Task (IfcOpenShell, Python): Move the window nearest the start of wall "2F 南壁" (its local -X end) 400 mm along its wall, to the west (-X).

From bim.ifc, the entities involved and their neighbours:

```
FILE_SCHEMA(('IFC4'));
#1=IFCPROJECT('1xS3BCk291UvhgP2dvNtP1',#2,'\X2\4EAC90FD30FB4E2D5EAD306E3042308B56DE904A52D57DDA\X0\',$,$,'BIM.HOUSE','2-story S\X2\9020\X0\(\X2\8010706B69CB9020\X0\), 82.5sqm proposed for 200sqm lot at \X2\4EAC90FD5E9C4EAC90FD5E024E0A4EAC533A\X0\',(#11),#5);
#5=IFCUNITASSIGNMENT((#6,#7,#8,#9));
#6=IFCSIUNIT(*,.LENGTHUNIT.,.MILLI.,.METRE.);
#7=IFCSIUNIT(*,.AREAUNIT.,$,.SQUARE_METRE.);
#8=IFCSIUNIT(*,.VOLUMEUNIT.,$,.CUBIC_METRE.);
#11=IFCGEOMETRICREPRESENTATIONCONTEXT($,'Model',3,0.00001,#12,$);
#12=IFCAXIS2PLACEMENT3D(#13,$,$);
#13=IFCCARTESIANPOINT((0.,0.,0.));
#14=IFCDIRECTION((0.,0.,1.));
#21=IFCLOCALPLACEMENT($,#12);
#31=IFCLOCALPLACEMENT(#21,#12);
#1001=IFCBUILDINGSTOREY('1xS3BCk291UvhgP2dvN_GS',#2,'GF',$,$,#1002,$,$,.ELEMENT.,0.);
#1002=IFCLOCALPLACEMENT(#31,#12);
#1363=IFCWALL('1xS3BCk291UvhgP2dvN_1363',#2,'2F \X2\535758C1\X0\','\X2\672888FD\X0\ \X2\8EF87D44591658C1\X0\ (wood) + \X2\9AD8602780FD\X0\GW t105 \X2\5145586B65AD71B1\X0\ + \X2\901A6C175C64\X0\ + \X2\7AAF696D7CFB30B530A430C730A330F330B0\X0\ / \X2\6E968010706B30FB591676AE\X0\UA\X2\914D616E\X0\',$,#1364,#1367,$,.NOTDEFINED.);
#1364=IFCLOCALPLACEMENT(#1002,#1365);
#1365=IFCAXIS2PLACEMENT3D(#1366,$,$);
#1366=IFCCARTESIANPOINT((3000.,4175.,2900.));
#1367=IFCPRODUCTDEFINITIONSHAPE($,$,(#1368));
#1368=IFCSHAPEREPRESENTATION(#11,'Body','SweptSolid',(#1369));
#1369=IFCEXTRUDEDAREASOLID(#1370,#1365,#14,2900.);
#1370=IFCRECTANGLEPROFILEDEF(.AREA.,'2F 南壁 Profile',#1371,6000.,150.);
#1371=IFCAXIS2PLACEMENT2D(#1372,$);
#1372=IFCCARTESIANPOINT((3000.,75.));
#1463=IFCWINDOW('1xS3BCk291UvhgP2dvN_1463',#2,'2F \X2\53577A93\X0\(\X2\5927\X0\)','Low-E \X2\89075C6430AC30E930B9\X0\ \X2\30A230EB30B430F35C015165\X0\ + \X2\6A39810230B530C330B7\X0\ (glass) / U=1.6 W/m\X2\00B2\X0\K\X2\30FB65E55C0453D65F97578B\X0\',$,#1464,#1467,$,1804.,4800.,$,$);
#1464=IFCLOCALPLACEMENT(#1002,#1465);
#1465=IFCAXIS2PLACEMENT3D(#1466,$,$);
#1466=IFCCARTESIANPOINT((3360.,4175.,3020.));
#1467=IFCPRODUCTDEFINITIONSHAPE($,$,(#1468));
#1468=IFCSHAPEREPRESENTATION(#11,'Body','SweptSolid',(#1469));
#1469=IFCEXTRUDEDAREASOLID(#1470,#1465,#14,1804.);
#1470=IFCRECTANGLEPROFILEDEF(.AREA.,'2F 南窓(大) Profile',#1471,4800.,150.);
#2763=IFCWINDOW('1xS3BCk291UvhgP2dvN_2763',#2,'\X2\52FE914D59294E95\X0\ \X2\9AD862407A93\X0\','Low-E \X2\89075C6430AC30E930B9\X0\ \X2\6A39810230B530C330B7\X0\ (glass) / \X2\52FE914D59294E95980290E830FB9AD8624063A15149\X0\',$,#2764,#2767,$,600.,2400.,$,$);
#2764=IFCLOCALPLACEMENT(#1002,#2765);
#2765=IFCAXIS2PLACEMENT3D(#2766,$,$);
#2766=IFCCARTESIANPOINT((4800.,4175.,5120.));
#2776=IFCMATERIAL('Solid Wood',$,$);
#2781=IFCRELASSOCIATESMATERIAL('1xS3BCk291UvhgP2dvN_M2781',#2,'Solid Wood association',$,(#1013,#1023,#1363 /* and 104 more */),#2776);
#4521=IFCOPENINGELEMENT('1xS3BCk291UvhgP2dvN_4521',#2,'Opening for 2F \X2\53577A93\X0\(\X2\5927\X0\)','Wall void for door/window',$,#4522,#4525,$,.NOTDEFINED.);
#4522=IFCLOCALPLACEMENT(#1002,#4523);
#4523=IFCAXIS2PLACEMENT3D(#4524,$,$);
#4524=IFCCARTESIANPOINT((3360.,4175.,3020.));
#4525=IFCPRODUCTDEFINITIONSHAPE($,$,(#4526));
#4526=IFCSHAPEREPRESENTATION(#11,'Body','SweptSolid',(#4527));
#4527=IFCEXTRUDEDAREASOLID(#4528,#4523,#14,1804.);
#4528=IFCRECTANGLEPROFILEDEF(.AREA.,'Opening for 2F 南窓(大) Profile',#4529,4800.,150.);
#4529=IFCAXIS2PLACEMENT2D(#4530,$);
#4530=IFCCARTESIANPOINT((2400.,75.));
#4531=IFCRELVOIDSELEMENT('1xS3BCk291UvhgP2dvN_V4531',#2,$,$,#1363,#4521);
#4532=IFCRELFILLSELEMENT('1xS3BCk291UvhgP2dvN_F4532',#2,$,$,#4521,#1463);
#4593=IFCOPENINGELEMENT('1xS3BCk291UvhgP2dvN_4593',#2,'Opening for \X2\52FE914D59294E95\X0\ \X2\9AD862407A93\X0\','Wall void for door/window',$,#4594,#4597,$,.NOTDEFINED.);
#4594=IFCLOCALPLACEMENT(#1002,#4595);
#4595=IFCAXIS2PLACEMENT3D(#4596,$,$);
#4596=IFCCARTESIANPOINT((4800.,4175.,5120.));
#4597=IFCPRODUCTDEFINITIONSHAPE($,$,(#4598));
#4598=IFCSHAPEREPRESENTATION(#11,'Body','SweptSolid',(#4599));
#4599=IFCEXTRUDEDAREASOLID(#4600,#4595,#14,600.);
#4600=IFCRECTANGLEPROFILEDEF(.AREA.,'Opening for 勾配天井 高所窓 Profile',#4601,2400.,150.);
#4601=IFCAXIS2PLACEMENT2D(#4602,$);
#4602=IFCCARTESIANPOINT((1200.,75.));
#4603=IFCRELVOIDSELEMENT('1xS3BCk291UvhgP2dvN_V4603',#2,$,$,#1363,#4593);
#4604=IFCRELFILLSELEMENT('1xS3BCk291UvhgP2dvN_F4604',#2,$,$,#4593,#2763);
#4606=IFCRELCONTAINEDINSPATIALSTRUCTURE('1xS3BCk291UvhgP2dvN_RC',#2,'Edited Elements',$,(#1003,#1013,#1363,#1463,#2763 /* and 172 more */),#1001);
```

```python
import ifcopenshell
import ifcopenshell.api.geometry
import ifcopenshell.util.placement

model = ifcopenshell.open("bim.ifc")

window = model.by_guid("1xS3BCk291UvhgP2dvN_1463")
opening = window.FillsVoids[0].RelatingOpeningElement
wall = opening.VoidsElements[0].RelatingBuildingElement

wall_matrix = ifcopenshell.util.placement.get_local_placement(wall.ObjectPlacement)
shift = wall_matrix[:3, 0] * -400.0
before = ifcopenshell.util.placement.get_local_placement(window.ObjectPlacement)[:3, 3].copy()

# The window is not placed relative to its opening, so move both.
for product in (opening, window):
    matrix = ifcopenshell.util.placement.get_local_placement(product.ObjectPlacement)
    matrix[:3, 3] += shift
    ifcopenshell.api.geometry.edit_object_placement(model, product=product, matrix=matrix, is_si=False)

after = ifcopenshell.util.placement.get_local_placement(window.ObjectPlacement)[:3, 3]
print("window moved by", (after - before).round(3) + 0.0)

model.write("bim_edited.ifc")
```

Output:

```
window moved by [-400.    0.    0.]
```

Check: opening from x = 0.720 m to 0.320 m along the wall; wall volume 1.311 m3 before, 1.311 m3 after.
